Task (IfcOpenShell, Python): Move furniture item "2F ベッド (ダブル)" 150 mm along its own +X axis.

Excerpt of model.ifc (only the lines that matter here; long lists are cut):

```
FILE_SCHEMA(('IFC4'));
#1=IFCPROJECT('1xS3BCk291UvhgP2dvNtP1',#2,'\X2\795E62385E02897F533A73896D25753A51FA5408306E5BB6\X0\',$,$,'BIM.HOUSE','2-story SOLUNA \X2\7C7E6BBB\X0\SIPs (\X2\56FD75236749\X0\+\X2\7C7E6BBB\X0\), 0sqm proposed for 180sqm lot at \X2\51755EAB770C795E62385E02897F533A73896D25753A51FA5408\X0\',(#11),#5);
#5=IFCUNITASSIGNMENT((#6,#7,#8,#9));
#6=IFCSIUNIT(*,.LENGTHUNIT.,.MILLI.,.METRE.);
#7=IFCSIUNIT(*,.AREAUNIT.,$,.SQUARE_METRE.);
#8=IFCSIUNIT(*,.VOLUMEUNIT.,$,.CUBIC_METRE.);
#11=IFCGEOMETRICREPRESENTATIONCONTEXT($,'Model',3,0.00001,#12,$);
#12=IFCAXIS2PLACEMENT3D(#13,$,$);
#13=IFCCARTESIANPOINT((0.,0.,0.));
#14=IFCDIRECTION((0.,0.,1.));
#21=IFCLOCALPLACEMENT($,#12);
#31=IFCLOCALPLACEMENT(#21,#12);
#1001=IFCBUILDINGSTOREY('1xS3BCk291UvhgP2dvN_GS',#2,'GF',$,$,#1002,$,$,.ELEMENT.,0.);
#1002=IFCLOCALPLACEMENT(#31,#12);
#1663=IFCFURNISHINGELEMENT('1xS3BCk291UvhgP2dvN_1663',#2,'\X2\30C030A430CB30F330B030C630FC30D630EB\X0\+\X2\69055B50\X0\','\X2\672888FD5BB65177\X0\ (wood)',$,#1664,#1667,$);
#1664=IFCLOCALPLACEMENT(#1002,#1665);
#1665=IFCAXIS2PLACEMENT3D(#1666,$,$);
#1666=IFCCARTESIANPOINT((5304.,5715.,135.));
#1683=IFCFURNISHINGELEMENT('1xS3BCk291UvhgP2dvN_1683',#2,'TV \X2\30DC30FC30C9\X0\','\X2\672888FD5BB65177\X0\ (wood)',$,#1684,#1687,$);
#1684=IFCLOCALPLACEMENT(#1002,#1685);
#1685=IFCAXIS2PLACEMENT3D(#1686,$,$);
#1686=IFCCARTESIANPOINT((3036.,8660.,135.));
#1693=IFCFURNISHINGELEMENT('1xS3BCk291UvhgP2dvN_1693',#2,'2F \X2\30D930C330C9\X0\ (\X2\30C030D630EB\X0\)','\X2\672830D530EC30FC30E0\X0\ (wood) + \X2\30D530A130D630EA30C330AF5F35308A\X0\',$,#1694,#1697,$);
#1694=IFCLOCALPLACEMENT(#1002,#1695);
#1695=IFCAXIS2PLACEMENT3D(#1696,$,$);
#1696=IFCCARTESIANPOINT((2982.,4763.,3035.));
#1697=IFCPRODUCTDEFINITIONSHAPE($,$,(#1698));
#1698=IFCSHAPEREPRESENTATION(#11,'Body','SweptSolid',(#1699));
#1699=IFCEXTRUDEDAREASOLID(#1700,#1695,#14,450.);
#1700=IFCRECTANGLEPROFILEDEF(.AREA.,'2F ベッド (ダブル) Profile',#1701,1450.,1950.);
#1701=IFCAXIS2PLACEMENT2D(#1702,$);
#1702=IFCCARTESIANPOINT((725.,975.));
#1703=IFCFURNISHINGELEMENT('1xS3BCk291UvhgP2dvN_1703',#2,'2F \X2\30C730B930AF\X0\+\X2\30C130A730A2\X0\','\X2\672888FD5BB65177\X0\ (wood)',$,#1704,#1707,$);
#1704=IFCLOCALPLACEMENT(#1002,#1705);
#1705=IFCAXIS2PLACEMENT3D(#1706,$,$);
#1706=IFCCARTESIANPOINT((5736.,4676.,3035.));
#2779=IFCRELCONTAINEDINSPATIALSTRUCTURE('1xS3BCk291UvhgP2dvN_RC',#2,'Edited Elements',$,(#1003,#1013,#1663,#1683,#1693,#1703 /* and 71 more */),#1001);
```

```python
import ifcopenshell
import ifcopenshell.api.geometry
import ifcopenshell.util.placement
import ifcopenshell.util.unit

model = ifcopenshell.open("model.ifc")
unit_scale = ifcopenshell.util.unit.calculate_unit_scale(model)

item = model.by_guid("1xS3BCk291UvhgP2dvN_1693")
matrix = ifcopenshell.util.placement.get_local_placement(item.ObjectPlacement)
matrix[:3, 3] += matrix[:3, 0] * 0.15 / unit_scale
ifcopenshell.api.geometry.edit_object_placement(model, product=item, matrix=matrix, is_si=False)

print(ifcopenshell.util.placement.get_local_placement(item.ObjectPlacement).round(3) + 0.0)

model.write("model_rev.ifc")
```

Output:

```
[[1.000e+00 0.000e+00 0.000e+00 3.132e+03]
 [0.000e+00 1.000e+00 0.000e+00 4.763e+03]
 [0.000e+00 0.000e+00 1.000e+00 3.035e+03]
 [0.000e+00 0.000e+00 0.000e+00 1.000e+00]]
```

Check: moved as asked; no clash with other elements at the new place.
